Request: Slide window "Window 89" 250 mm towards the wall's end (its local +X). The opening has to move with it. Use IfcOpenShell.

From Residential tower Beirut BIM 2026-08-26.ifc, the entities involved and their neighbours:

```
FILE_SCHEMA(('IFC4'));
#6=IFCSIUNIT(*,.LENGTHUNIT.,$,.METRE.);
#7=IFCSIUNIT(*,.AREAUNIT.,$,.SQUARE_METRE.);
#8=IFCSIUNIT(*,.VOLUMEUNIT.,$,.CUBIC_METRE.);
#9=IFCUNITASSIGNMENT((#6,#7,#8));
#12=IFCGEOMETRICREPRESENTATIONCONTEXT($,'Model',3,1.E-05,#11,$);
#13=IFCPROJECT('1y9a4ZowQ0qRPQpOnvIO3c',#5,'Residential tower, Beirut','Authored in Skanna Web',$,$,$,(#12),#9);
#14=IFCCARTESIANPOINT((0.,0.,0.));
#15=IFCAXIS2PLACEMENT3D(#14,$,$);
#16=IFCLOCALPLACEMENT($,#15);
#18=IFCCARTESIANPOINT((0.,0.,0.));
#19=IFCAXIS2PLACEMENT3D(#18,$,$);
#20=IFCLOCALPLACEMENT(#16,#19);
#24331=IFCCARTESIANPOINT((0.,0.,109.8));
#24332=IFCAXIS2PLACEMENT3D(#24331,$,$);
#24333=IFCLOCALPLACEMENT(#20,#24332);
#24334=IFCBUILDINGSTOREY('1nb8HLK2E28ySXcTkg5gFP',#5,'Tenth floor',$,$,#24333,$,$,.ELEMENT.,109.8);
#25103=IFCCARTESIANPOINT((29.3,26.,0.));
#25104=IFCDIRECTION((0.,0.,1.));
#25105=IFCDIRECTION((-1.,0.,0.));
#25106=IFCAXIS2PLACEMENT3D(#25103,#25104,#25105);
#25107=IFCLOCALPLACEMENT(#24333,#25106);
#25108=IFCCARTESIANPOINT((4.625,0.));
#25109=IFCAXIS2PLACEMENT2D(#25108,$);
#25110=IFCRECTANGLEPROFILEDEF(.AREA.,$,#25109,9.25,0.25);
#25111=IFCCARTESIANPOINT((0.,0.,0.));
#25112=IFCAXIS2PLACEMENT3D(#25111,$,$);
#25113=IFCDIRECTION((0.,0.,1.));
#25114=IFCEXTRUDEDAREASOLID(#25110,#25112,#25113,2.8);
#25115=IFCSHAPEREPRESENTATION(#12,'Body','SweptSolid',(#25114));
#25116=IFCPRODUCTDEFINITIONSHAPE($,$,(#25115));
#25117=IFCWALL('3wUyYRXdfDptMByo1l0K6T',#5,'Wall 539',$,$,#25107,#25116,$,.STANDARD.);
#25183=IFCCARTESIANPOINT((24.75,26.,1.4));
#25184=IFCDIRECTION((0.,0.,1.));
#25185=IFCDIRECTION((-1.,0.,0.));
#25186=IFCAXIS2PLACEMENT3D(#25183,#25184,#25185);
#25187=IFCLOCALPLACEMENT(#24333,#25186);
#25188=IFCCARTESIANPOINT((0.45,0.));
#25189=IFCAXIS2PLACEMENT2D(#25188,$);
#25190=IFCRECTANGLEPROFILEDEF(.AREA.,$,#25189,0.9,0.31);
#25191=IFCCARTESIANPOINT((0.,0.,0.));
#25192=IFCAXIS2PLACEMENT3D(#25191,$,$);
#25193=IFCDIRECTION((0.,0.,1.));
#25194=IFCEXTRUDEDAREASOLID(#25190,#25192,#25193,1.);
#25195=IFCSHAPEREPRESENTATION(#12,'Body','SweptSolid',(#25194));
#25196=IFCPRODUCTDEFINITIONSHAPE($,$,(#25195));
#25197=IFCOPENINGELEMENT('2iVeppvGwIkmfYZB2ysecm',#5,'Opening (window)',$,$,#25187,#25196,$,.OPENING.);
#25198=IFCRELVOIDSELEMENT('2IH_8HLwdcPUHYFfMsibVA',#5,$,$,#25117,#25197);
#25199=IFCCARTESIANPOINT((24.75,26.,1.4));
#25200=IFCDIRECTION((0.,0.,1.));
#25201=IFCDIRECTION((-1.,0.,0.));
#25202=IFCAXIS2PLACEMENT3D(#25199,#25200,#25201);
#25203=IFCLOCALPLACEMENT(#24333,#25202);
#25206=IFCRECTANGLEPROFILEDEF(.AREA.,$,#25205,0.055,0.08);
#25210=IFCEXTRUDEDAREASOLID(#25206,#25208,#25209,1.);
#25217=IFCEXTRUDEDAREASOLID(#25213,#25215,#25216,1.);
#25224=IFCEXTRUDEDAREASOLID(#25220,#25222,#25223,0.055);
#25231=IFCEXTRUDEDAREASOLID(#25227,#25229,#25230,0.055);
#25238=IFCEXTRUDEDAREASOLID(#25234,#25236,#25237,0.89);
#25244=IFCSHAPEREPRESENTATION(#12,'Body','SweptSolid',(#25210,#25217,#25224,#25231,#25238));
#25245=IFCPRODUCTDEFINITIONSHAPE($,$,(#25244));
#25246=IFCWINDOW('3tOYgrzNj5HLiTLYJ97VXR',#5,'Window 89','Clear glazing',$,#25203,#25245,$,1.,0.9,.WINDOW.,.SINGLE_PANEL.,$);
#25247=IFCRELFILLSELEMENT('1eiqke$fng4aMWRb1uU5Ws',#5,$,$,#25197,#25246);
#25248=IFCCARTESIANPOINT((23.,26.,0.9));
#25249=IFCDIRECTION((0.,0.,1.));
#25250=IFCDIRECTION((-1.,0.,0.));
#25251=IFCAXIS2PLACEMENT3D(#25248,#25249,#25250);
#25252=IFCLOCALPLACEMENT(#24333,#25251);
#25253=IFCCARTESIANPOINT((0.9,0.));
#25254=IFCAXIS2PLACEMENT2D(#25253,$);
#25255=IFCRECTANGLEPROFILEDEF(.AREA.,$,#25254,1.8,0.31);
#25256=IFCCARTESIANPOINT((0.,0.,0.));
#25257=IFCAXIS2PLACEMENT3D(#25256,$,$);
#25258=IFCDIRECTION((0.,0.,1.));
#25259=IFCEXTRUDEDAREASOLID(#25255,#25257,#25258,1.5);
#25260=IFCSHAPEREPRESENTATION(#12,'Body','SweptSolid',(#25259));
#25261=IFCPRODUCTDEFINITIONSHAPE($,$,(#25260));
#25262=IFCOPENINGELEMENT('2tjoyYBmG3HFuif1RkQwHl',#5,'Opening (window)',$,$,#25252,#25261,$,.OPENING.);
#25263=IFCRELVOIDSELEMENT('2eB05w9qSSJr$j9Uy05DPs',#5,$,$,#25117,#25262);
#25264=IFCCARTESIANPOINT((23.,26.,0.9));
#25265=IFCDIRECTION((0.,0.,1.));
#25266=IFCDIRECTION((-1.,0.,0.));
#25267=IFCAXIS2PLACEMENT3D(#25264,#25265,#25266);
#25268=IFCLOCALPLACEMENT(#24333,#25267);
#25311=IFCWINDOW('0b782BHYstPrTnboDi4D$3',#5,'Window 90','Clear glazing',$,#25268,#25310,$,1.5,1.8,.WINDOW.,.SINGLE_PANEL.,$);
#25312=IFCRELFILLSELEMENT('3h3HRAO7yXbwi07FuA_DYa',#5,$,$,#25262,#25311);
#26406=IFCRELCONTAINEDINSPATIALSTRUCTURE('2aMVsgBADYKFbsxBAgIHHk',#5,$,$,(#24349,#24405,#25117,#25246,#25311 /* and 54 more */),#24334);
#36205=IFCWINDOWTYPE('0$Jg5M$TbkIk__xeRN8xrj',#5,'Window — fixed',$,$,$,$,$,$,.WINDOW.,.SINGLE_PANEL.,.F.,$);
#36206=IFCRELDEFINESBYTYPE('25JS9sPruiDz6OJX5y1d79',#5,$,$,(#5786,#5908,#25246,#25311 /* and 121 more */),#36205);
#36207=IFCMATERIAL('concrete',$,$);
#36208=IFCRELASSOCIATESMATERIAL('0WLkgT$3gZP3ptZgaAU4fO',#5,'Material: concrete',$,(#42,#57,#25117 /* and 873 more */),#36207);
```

```python
import ifcopenshell
import ifcopenshell.api.geometry
import ifcopenshell.util.placement

model = ifcopenshell.open("Residential tower Beirut BIM 2026-08-26.ifc")

window = model.by_id(25246)
opening = window.FillsVoids[0].RelatingOpeningElement
wall = opening.VoidsElements[0].RelatingBuildingElement

wall_matrix = ifcopenshell.util.placement.get_local_placement(wall.ObjectPlacement)
shift = wall_matrix[:3, 0] * 0.25
before = ifcopenshell.util.placement.get_local_placement(window.ObjectPlacement)[:3, 3].copy()

# The window is not placed relative to its opening, so move both.
for product in (opening, window):
    matrix = ifcopenshell.util.placement.get_local_placement(product.ObjectPlacement)
    matrix[:3, 3] += shift
    ifcopenshell.api.geometry.edit_object_placement(model, product=product, matrix=matrix, is_si=False)

after = ifcopenshell.util.placement.get_local_placement(window.ObjectPlacement)[:3, 3]
print("window moved by", (after - before).round(3) + 0.0)

model.write("Residential tower Beirut BIM 2026-08-26_v2.ifc")
```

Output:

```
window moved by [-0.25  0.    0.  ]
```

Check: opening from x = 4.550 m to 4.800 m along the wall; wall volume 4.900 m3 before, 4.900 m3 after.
